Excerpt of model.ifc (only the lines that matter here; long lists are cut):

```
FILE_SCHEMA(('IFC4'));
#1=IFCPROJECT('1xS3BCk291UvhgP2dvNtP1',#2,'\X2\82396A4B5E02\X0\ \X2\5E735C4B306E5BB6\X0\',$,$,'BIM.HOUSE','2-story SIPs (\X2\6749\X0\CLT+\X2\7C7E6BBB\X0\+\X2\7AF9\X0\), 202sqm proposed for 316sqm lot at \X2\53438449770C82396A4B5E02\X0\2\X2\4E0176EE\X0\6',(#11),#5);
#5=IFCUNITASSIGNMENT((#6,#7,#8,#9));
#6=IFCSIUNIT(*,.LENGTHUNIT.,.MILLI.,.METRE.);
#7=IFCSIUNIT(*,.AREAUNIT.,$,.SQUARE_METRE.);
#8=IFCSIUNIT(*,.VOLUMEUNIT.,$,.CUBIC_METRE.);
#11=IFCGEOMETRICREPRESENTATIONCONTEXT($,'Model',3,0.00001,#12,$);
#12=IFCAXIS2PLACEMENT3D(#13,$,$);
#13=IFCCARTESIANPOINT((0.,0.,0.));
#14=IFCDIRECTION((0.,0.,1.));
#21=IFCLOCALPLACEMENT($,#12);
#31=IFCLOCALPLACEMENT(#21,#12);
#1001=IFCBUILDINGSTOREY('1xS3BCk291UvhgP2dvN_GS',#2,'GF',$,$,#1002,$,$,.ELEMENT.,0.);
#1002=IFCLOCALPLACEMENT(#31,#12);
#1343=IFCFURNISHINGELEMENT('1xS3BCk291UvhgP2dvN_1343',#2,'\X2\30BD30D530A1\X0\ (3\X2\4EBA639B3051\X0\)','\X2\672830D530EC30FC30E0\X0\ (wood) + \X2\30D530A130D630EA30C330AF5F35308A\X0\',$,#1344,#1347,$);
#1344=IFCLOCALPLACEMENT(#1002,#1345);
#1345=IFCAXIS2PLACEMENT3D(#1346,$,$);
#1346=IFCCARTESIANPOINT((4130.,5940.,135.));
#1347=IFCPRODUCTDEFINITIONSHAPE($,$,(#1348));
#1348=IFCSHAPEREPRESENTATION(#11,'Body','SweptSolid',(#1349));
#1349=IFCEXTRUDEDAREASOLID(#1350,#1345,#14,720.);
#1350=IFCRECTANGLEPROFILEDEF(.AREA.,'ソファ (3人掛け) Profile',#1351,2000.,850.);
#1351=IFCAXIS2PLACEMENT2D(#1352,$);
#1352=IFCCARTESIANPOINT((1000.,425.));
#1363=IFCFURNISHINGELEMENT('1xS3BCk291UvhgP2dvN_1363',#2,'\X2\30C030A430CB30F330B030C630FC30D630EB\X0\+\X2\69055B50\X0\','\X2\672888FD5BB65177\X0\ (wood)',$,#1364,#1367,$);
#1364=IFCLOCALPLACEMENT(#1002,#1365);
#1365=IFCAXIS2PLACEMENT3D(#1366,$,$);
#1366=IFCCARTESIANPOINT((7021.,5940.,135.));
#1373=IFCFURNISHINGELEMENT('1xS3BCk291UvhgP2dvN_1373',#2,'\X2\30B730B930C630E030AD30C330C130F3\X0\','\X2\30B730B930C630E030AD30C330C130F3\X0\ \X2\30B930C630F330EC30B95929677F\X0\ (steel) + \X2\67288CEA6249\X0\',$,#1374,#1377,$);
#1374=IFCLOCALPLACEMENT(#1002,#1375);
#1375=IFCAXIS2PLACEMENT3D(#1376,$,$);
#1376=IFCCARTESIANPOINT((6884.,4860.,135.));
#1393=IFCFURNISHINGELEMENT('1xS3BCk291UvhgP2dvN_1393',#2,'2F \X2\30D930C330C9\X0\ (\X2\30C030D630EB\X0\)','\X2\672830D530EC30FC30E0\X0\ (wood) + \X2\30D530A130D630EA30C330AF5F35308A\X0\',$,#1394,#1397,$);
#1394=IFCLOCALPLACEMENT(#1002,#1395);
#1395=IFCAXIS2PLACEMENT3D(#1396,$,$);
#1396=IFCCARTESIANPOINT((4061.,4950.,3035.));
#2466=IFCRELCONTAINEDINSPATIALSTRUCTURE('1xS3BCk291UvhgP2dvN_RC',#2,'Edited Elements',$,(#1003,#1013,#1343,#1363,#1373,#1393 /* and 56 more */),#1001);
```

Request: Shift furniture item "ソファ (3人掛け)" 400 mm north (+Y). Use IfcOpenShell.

```python
import ifcopenshell
import ifcopenshell.api.geometry
import ifcopenshell.util.placement

model = ifcopenshell.open("model.ifc")

item = model.by_id(1343)
matrix = ifcopenshell.util.placement.get_local_placement(item.ObjectPlacement)
matrix[1, 3] += 400.0
ifcopenshell.api.geometry.edit_object_placement(model, product=item, matrix=matrix, is_si=False)

print(ifcopenshell.util.placement.get_local_placement(item.ObjectPlacement).round(3) + 0.0)

model.write("model_edited.ifc")
```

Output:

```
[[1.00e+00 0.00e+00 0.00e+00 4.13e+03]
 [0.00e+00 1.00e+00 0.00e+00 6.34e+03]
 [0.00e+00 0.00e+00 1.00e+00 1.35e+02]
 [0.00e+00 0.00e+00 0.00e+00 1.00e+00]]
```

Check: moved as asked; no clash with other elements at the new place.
